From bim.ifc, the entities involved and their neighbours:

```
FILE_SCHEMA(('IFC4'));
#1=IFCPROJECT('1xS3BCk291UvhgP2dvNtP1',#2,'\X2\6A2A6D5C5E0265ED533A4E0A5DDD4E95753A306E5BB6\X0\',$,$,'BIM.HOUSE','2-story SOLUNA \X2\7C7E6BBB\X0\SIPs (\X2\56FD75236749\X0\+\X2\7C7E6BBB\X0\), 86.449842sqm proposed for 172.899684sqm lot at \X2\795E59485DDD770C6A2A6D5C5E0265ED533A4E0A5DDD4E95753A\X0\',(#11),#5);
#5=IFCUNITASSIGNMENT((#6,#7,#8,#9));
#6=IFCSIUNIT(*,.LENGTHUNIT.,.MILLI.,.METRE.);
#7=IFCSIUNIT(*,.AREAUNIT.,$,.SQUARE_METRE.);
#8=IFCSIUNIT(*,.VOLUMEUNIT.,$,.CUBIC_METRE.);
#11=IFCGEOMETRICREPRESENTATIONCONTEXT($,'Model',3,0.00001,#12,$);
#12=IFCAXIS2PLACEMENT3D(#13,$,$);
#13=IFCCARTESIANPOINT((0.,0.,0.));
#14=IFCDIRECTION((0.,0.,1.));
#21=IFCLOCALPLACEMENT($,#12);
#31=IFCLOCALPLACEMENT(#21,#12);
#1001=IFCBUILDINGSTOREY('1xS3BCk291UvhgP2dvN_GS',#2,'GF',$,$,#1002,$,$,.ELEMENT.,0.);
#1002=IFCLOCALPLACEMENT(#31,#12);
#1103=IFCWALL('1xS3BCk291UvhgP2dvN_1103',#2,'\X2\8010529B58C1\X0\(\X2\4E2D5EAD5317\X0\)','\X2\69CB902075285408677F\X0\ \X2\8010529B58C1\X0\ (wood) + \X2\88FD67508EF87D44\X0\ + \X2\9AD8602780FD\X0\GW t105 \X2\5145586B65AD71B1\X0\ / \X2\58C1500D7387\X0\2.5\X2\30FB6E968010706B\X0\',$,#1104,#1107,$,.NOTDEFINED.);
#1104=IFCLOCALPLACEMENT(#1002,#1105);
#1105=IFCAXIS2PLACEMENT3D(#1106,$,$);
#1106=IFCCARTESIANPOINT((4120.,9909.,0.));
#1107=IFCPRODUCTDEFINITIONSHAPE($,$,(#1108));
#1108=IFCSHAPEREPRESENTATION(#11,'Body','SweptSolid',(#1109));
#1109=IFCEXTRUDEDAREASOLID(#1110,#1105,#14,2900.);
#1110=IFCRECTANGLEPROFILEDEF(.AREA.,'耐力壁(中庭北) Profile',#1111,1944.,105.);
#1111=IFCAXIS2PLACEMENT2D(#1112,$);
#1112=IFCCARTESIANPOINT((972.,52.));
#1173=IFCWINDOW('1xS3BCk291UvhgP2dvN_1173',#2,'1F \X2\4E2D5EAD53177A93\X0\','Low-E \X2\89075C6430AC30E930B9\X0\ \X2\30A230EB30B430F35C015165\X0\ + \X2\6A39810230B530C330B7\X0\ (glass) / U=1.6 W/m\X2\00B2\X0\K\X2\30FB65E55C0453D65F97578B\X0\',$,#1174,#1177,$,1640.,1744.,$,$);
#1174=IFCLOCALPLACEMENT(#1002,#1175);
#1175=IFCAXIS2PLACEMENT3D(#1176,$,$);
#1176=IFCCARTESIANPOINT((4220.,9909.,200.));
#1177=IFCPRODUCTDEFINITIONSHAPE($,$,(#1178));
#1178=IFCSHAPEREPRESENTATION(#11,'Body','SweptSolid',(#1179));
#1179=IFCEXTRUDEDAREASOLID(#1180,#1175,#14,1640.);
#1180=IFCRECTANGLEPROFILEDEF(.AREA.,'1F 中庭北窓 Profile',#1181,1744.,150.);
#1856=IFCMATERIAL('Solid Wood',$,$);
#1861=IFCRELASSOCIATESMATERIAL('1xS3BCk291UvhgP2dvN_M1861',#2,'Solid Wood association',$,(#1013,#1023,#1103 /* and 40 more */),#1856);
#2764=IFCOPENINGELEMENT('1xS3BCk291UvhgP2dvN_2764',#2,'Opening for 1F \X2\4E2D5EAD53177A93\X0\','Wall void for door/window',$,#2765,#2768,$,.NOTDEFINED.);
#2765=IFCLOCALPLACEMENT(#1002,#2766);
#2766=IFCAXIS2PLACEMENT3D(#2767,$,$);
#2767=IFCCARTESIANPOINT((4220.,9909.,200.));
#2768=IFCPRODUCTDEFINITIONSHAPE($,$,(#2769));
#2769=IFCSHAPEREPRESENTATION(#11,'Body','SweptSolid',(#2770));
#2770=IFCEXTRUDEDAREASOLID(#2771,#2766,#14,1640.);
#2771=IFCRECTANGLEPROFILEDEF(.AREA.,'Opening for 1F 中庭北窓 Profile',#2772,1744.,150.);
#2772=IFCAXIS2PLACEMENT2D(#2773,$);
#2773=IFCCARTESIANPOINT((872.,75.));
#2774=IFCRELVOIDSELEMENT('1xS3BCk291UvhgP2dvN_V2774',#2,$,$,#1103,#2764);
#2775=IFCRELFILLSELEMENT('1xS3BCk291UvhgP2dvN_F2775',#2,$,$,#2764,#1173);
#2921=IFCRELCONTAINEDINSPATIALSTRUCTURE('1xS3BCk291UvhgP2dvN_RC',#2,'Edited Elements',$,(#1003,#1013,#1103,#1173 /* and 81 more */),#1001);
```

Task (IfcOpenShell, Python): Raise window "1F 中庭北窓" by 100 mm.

```python
import numpy as np
import ifcopenshell
import ifcopenshell.api.geometry
import ifcopenshell.util.placement
import ifcopenshell.util.unit

model = ifcopenshell.open("bim.ifc")
unit_scale = ifcopenshell.util.unit.calculate_unit_scale(model)

window = model.by_guid("1xS3BCk291UvhgP2dvN_1173")
opening = window.FillsVoids[0].RelatingOpeningElement
dz = 100.0

shift = np.array([0.0, 0.0, dz])
# The window is not placed relative to its opening, so move both.
for product in (opening, window):
    matrix = ifcopenshell.util.placement.get_local_placement(product.ObjectPlacement)
    matrix[:3, 3] += shift
    ifcopenshell.api.geometry.edit_object_placement(model, product=product, matrix=matrix, is_si=False)

print(f"moved by {dz * unit_scale:+.3f} m")

model.write("bim_updated.ifc")
```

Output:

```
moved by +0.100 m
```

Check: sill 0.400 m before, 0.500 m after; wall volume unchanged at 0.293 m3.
